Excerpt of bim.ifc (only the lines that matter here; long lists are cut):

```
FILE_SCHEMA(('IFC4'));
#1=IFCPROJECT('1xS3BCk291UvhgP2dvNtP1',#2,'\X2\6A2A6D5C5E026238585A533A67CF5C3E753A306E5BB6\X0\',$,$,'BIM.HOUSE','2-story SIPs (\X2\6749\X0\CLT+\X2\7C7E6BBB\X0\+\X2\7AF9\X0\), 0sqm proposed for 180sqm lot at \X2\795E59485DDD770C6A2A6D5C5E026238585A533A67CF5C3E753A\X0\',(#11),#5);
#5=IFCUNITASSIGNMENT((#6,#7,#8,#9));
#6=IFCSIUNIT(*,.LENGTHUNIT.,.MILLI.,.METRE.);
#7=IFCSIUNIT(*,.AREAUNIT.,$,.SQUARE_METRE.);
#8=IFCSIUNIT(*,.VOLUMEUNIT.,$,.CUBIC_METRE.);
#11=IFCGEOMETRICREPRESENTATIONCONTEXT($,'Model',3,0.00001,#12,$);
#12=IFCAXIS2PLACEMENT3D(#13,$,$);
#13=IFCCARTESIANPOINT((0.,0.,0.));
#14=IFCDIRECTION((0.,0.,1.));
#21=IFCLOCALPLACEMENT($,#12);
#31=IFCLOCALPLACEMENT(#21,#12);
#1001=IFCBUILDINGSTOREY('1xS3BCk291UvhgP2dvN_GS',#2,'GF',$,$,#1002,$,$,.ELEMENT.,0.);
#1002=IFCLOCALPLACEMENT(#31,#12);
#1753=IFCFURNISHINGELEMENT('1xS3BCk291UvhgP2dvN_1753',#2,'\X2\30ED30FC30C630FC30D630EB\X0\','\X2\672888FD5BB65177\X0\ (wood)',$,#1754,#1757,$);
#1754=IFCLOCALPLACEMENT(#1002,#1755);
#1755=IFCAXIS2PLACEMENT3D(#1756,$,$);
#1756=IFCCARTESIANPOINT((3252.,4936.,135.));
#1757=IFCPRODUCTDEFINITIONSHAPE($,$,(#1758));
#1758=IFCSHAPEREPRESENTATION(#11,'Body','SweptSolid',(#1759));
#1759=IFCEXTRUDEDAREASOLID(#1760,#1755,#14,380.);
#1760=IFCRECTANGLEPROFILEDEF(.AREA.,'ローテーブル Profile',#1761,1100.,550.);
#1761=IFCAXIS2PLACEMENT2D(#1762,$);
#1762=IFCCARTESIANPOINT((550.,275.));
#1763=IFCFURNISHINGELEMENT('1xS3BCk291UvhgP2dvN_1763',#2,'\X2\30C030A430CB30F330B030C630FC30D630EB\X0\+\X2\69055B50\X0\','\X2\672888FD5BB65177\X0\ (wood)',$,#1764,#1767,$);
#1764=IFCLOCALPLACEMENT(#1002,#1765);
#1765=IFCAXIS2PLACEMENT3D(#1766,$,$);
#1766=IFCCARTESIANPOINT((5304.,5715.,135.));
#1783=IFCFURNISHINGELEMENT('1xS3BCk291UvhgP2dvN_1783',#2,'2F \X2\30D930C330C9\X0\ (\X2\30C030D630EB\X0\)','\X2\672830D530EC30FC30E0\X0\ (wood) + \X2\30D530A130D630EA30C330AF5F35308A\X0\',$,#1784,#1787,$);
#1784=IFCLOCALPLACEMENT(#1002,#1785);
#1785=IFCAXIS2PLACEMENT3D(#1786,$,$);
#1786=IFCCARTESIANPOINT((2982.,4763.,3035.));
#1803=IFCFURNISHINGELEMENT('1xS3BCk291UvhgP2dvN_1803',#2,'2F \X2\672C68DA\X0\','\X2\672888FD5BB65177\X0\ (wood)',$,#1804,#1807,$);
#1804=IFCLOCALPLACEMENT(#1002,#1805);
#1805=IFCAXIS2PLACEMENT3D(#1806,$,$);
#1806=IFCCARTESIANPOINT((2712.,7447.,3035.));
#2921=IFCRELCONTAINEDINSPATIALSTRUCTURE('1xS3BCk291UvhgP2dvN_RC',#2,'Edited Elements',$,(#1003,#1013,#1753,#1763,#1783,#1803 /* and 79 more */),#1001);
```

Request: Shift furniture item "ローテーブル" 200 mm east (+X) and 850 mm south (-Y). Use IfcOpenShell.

```python
import ifcopenshell
import ifcopenshell.api.geometry
import ifcopenshell.util.placement
import ifcopenshell.util.unit

model = ifcopenshell.open("bim.ifc")
unit_scale = ifcopenshell.util.unit.calculate_unit_scale(model)

item = model.by_id(1753)
matrix = ifcopenshell.util.placement.get_local_placement(item.ObjectPlacement)
matrix[0, 3] += 0.2 / unit_scale
matrix[1, 3] -= 0.85 / unit_scale
ifcopenshell.api.geometry.edit_object_placement(model, product=item, matrix=matrix, is_si=False)

print(ifcopenshell.util.placement.get_local_placement(item.ObjectPlacement).round(3) + 0.0)

model.write("bim_edited.ifc")
```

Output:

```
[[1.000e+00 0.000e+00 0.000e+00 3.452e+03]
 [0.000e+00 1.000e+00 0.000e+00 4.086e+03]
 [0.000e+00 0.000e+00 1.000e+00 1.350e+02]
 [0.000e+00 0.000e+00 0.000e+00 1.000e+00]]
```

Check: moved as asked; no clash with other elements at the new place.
